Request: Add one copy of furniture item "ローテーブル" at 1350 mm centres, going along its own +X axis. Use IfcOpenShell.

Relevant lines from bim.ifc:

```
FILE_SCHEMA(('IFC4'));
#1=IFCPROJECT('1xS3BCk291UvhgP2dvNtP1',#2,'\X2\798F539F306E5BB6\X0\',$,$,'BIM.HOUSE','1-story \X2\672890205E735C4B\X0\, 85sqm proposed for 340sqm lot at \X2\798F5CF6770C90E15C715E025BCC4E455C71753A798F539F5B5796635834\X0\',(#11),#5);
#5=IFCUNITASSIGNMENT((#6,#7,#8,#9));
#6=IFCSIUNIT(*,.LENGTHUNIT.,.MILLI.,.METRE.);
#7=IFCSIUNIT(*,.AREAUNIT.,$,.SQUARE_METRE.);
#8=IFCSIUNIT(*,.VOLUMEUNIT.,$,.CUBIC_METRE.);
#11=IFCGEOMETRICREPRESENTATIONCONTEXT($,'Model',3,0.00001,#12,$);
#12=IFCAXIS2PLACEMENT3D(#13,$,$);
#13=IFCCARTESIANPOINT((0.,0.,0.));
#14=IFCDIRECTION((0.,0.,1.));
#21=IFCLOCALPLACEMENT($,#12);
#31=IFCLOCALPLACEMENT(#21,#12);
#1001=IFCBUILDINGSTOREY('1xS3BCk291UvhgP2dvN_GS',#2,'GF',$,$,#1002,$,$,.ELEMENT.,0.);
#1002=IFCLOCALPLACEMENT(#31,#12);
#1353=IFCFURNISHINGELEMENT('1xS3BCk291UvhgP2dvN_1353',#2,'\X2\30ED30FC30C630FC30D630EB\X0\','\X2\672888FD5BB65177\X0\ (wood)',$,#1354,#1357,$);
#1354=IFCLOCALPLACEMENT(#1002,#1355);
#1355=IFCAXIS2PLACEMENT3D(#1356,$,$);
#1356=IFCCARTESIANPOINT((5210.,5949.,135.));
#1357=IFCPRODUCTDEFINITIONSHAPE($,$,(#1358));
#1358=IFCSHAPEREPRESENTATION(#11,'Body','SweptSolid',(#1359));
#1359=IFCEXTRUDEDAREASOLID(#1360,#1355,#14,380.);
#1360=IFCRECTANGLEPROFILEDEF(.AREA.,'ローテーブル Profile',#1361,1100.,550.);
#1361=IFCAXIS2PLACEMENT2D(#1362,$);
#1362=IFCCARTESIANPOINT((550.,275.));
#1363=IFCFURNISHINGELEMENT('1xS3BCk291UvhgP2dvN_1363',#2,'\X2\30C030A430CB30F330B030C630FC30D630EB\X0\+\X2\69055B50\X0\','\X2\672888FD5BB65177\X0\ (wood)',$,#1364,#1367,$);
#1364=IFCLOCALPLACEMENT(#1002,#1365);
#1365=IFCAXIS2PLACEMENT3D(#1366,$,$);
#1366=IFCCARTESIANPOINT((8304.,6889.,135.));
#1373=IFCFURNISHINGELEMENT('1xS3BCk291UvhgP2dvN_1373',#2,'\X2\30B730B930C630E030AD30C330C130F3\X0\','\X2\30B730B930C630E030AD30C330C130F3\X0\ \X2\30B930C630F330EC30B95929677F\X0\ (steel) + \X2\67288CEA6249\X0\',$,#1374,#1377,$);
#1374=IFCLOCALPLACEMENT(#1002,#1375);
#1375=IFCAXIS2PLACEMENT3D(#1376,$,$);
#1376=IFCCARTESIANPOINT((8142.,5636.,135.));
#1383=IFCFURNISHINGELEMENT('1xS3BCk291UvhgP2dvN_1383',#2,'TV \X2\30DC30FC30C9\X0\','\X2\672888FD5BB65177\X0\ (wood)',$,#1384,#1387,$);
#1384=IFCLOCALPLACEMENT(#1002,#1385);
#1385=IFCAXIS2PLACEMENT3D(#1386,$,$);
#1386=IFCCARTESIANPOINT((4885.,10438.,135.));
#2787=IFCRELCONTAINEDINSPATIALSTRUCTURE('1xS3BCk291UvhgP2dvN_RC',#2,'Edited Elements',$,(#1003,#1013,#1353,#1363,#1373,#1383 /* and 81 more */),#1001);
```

```python
import ifcopenshell
import ifcopenshell.api.geometry
import ifcopenshell.api.root
import ifcopenshell.util.element
import ifcopenshell.util.placement
import ifcopenshell.util.unit

model = ifcopenshell.open("bim.ifc")
unit_scale = ifcopenshell.util.unit.calculate_unit_scale(model)


def reuse_history(source, copy):
    """copy_class also copies each property set's owner history, people and application; keep the originals."""
    for rel in copy.IsDefinedBy:
        if rel.is_a("IfcRelDefinesByProperties") and (history := rel.RelatingPropertyDefinition.OwnerHistory):
            rel.RelatingPropertyDefinition.OwnerHistory = source.OwnerHistory
            ifcopenshell.util.element.remove_deep2(model, history)


source = model.by_id(1353)
base = ifcopenshell.util.placement.get_local_placement(source.ObjectPlacement)
step = base[:3, 0] * 1.35 / unit_scale

for i in range(1, 2):
    copy = ifcopenshell.api.root.copy_class(model, product=source)
    copy.Representation = ifcopenshell.util.element.copy_deep(
        model, source.Representation, exclude=["IfcGeometricRepresentationContext", "IfcRepresentationMap"]
    )
    reuse_history(source, copy)
    matrix = base.copy()
    matrix[:3, 3] += i * step
    print("added at", matrix[:3, 3].round(3) + 0.0)
    ifcopenshell.api.geometry.edit_object_placement(model, product=copy, matrix=matrix, is_si=False)

model.write("bim_v2.ifc")
```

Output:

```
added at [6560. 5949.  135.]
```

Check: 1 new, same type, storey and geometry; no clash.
